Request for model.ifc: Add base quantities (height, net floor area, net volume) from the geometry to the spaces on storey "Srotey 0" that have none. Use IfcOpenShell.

First a look at what the model holds.

```python
import ifcopenshell
import ifcopenshell.util.element
import ifcopenshell.util.unit

model = ifcopenshell.open("model.ifc")
print(model.schema)
for unit_type in ("LENGTHUNIT", "AREAUNIT", "VOLUMEUNIT"):
    print(unit_type, ifcopenshell.util.unit.calculate_unit_scale(model, unit_type))
storey = next(s for s in model.by_type("IfcBuildingStorey") if s.Name == "Srotey 0")
spaces = [e for e in ifcopenshell.util.element.get_decomposition(storey) if e.is_a("IfcSpace")]
for e in sorted(spaces, key=lambda e: e.id()):
    print(e.id(), e.is_a(), e.Name, list(ifcopenshell.util.element.get_psets(e, qtos_only=True)), sep=" | ")
```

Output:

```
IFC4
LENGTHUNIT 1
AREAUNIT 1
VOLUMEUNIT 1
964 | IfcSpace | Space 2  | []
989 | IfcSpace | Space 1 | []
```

```python
import ifcopenshell
import ifcopenshell.api.pset
import ifcopenshell.geom
import ifcopenshell.util.element
import ifcopenshell.util.shape
import ifcopenshell.util.unit

model = ifcopenshell.open("model.ifc")
unit_scale = ifcopenshell.util.unit.calculate_unit_scale(model)
area_scale = ifcopenshell.util.unit.calculate_unit_scale(model, "AREAUNIT")
volume_scale = ifcopenshell.util.unit.calculate_unit_scale(model, "VOLUMEUNIT")
settings = ifcopenshell.geom.settings()

storey = next(s for s in model.by_type("IfcBuildingStorey") if s.Name == "Srotey 0")
spaces = [e for e in ifcopenshell.util.element.get_decomposition(storey) if e.is_a("IfcSpace")]

for e in sorted(spaces, key=lambda e: e.id()):
    if ifcopenshell.util.element.get_psets(e, qtos_only=True, should_inherit=False):
        continue
    # Geometry comes back in metres, in the element's own axes.
    shape = ifcopenshell.geom.create_shape(settings, e)
    values = {
        "Height": ifcopenshell.util.shape.get_z(shape.geometry) / unit_scale,
        "NetFloorArea": ifcopenshell.util.shape.get_footprint_area(shape.geometry) / area_scale,
        "NetVolume": ifcopenshell.util.shape.get_volume(shape.geometry) / volume_scale,
    }
    qto = ifcopenshell.api.pset.add_qto(model, product=e, name="Qto_SpaceBaseQuantities")
    ifcopenshell.api.pset.edit_qto(model, qto=qto, properties=values)
    print(e.id(), {k: round(v, 3) for k, v in values.items()})

model.write("model_updated.ifc")
```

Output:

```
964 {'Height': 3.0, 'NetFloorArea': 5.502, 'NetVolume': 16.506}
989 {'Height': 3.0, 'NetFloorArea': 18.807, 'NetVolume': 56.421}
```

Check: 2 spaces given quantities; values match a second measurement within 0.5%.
